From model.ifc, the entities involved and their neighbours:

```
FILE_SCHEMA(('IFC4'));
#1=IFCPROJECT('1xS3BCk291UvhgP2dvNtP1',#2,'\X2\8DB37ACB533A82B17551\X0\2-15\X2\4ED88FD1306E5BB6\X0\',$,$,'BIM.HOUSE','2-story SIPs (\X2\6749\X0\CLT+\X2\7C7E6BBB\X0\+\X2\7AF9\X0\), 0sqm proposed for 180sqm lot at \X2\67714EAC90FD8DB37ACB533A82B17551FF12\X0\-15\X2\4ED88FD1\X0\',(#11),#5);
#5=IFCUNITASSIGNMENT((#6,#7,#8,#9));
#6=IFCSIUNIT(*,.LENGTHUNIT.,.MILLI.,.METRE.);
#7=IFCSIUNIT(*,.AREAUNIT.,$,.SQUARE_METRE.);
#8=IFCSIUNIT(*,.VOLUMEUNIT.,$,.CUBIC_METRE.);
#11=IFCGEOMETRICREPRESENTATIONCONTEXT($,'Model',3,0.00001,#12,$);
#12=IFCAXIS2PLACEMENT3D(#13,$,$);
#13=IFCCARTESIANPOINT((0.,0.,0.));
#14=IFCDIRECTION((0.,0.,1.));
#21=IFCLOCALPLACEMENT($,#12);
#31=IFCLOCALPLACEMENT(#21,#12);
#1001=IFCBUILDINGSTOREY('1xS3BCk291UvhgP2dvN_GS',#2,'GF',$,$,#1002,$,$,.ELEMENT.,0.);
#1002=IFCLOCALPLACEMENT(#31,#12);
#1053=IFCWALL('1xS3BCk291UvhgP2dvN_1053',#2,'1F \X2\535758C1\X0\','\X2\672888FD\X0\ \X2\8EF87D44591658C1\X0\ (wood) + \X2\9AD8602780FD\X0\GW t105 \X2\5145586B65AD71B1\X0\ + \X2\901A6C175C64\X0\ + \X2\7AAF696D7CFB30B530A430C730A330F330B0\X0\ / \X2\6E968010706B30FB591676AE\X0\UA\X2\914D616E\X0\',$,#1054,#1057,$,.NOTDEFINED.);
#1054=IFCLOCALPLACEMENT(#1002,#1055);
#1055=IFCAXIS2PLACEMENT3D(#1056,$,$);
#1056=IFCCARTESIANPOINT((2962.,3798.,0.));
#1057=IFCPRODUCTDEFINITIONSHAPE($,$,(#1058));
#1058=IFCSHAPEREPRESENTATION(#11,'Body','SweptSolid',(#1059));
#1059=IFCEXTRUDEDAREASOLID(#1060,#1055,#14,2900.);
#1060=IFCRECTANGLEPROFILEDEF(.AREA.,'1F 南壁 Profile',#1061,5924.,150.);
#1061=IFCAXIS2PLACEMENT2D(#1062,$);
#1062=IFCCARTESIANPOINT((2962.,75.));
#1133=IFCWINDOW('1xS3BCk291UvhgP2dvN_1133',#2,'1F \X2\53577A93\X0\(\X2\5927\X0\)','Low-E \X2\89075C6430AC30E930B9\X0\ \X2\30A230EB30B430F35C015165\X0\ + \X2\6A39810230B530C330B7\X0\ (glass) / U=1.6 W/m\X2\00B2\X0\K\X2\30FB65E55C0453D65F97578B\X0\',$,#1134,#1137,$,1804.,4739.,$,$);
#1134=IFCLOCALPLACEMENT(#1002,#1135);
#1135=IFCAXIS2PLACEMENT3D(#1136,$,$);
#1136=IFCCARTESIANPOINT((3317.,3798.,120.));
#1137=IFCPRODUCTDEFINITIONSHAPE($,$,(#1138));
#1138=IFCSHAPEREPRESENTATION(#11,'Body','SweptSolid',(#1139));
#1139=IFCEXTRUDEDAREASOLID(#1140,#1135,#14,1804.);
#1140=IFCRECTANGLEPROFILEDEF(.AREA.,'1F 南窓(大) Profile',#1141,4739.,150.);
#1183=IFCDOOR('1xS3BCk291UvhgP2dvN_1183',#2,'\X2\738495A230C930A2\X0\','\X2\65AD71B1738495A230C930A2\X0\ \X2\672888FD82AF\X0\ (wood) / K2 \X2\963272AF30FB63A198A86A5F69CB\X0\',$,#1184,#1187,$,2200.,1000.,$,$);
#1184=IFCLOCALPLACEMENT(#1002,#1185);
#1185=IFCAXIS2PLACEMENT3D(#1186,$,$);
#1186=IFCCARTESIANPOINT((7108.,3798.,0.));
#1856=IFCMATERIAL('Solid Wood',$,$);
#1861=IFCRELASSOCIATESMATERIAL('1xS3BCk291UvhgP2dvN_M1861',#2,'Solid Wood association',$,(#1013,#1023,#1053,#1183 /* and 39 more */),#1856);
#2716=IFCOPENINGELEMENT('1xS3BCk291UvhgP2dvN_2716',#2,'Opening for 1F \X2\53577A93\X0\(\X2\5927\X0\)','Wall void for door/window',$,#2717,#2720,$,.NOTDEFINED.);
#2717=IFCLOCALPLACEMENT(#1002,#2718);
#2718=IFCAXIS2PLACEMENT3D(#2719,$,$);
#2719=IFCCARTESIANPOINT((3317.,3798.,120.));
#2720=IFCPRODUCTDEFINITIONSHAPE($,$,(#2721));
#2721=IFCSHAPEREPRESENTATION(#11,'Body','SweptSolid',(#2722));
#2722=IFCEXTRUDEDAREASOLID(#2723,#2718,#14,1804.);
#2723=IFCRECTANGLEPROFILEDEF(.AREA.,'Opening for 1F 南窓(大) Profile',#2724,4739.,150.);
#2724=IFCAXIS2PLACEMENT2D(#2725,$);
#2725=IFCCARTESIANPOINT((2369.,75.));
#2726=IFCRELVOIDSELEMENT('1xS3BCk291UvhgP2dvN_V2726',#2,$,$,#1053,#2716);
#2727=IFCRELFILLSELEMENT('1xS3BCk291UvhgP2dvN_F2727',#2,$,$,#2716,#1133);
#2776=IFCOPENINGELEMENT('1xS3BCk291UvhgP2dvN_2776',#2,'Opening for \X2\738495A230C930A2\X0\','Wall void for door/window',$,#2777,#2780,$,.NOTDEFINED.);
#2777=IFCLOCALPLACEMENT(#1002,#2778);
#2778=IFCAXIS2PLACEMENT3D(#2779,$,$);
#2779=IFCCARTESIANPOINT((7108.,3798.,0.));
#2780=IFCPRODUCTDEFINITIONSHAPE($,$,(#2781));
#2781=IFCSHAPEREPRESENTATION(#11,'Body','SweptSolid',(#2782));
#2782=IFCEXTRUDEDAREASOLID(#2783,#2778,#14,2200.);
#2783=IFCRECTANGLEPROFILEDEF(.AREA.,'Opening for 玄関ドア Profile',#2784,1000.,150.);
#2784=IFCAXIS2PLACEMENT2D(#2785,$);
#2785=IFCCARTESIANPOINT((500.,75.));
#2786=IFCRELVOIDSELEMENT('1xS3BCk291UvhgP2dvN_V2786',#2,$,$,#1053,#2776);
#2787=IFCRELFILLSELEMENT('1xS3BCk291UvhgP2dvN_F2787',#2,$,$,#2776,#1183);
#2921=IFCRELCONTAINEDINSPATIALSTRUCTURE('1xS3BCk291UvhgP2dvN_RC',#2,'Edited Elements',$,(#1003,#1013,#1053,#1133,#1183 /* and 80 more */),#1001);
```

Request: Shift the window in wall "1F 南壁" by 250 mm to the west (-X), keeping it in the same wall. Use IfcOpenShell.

```python
import ifcopenshell
import ifcopenshell.api.geometry
import ifcopenshell.util.placement

model = ifcopenshell.open("model.ifc")

window = model.by_guid("1xS3BCk291UvhgP2dvN_1133")
opening = window.FillsVoids[0].RelatingOpeningElement
wall = opening.VoidsElements[0].RelatingBuildingElement

wall_matrix = ifcopenshell.util.placement.get_local_placement(wall.ObjectPlacement)
shift = wall_matrix[:3, 0] * -250.0
before = ifcopenshell.util.placement.get_local_placement(window.ObjectPlacement)[:3, 3].copy()

# The window is not placed relative to its opening, so move both.
for product in (opening, window):
    matrix = ifcopenshell.util.placement.get_local_placement(product.ObjectPlacement)
    matrix[:3, 3] += shift
    ifcopenshell.api.geometry.edit_object_placement(model, product=product, matrix=matrix, is_si=False)

after = ifcopenshell.util.placement.get_local_placement(window.ObjectPlacement)[:3, 3]
print("window moved by", (after - before).round(3) + 0.0)

model.write("model-out.ifc")
```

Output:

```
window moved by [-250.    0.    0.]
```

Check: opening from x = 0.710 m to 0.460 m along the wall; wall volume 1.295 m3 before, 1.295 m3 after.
